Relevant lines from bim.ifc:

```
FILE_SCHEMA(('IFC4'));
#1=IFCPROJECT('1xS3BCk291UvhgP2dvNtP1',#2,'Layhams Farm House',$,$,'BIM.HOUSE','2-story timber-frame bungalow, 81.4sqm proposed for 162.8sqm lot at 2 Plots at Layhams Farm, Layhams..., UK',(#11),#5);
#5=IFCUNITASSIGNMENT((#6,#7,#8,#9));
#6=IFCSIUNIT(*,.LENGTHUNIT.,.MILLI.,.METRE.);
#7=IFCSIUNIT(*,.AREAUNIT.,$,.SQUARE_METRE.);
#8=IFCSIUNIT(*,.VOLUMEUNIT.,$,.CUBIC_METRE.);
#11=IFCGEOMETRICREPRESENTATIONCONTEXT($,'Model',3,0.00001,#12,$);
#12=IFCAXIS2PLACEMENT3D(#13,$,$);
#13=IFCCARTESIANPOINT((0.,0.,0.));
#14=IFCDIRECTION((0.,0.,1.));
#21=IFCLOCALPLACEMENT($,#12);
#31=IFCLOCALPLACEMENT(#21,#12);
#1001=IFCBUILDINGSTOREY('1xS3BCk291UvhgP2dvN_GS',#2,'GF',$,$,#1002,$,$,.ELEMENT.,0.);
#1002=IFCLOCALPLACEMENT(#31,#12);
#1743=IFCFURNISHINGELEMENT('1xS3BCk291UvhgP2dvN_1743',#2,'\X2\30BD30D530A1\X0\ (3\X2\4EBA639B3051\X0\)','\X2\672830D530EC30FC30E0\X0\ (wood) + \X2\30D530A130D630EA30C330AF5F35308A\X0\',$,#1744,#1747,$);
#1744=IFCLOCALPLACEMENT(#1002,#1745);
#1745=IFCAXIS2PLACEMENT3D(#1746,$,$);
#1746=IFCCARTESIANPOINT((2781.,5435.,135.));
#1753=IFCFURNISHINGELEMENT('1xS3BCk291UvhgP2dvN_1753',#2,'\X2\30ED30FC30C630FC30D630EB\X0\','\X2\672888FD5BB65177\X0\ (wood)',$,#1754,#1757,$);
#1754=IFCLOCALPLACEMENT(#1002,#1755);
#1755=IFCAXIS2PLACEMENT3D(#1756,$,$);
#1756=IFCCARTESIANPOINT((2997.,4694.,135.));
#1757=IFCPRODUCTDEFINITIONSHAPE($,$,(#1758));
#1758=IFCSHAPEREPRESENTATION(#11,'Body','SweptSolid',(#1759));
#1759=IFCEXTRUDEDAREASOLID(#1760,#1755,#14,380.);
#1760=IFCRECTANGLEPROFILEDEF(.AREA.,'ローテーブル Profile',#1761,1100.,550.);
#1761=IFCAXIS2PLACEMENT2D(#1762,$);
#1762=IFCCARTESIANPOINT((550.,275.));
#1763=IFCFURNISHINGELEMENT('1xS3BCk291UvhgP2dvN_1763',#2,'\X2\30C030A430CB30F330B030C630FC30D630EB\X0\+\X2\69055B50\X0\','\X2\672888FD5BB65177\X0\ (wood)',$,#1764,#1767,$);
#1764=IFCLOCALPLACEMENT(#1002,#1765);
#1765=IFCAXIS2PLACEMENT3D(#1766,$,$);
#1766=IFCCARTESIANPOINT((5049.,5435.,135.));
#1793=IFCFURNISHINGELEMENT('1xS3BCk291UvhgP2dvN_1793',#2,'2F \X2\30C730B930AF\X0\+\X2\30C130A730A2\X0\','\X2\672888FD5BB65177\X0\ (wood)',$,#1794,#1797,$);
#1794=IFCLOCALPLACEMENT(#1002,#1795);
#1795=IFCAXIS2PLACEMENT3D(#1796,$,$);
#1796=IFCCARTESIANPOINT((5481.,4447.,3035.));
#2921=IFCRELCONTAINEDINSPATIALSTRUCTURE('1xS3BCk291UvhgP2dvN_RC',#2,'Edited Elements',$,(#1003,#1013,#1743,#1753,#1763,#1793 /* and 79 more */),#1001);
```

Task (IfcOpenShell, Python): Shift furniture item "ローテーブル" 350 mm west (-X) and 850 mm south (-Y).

```python
import ifcopenshell
import ifcopenshell.api.geometry
import ifcopenshell.util.placement

model = ifcopenshell.open("bim.ifc")

item = model.by_guid("1xS3BCk291UvhgP2dvN_1753")
matrix = ifcopenshell.util.placement.get_local_placement(item.ObjectPlacement)
matrix[0, 3] -= 350.0
matrix[1, 3] -= 850.0
ifcopenshell.api.geometry.edit_object_placement(model, product=item, matrix=matrix, is_si=False)

print(ifcopenshell.util.placement.get_local_placement(item.ObjectPlacement).round(3) + 0.0)

model.write("bim_rev.ifc")
```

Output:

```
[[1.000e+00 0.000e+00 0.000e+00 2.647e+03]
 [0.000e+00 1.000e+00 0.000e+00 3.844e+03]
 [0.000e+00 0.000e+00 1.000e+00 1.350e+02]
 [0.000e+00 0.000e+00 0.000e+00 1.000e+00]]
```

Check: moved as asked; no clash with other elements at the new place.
